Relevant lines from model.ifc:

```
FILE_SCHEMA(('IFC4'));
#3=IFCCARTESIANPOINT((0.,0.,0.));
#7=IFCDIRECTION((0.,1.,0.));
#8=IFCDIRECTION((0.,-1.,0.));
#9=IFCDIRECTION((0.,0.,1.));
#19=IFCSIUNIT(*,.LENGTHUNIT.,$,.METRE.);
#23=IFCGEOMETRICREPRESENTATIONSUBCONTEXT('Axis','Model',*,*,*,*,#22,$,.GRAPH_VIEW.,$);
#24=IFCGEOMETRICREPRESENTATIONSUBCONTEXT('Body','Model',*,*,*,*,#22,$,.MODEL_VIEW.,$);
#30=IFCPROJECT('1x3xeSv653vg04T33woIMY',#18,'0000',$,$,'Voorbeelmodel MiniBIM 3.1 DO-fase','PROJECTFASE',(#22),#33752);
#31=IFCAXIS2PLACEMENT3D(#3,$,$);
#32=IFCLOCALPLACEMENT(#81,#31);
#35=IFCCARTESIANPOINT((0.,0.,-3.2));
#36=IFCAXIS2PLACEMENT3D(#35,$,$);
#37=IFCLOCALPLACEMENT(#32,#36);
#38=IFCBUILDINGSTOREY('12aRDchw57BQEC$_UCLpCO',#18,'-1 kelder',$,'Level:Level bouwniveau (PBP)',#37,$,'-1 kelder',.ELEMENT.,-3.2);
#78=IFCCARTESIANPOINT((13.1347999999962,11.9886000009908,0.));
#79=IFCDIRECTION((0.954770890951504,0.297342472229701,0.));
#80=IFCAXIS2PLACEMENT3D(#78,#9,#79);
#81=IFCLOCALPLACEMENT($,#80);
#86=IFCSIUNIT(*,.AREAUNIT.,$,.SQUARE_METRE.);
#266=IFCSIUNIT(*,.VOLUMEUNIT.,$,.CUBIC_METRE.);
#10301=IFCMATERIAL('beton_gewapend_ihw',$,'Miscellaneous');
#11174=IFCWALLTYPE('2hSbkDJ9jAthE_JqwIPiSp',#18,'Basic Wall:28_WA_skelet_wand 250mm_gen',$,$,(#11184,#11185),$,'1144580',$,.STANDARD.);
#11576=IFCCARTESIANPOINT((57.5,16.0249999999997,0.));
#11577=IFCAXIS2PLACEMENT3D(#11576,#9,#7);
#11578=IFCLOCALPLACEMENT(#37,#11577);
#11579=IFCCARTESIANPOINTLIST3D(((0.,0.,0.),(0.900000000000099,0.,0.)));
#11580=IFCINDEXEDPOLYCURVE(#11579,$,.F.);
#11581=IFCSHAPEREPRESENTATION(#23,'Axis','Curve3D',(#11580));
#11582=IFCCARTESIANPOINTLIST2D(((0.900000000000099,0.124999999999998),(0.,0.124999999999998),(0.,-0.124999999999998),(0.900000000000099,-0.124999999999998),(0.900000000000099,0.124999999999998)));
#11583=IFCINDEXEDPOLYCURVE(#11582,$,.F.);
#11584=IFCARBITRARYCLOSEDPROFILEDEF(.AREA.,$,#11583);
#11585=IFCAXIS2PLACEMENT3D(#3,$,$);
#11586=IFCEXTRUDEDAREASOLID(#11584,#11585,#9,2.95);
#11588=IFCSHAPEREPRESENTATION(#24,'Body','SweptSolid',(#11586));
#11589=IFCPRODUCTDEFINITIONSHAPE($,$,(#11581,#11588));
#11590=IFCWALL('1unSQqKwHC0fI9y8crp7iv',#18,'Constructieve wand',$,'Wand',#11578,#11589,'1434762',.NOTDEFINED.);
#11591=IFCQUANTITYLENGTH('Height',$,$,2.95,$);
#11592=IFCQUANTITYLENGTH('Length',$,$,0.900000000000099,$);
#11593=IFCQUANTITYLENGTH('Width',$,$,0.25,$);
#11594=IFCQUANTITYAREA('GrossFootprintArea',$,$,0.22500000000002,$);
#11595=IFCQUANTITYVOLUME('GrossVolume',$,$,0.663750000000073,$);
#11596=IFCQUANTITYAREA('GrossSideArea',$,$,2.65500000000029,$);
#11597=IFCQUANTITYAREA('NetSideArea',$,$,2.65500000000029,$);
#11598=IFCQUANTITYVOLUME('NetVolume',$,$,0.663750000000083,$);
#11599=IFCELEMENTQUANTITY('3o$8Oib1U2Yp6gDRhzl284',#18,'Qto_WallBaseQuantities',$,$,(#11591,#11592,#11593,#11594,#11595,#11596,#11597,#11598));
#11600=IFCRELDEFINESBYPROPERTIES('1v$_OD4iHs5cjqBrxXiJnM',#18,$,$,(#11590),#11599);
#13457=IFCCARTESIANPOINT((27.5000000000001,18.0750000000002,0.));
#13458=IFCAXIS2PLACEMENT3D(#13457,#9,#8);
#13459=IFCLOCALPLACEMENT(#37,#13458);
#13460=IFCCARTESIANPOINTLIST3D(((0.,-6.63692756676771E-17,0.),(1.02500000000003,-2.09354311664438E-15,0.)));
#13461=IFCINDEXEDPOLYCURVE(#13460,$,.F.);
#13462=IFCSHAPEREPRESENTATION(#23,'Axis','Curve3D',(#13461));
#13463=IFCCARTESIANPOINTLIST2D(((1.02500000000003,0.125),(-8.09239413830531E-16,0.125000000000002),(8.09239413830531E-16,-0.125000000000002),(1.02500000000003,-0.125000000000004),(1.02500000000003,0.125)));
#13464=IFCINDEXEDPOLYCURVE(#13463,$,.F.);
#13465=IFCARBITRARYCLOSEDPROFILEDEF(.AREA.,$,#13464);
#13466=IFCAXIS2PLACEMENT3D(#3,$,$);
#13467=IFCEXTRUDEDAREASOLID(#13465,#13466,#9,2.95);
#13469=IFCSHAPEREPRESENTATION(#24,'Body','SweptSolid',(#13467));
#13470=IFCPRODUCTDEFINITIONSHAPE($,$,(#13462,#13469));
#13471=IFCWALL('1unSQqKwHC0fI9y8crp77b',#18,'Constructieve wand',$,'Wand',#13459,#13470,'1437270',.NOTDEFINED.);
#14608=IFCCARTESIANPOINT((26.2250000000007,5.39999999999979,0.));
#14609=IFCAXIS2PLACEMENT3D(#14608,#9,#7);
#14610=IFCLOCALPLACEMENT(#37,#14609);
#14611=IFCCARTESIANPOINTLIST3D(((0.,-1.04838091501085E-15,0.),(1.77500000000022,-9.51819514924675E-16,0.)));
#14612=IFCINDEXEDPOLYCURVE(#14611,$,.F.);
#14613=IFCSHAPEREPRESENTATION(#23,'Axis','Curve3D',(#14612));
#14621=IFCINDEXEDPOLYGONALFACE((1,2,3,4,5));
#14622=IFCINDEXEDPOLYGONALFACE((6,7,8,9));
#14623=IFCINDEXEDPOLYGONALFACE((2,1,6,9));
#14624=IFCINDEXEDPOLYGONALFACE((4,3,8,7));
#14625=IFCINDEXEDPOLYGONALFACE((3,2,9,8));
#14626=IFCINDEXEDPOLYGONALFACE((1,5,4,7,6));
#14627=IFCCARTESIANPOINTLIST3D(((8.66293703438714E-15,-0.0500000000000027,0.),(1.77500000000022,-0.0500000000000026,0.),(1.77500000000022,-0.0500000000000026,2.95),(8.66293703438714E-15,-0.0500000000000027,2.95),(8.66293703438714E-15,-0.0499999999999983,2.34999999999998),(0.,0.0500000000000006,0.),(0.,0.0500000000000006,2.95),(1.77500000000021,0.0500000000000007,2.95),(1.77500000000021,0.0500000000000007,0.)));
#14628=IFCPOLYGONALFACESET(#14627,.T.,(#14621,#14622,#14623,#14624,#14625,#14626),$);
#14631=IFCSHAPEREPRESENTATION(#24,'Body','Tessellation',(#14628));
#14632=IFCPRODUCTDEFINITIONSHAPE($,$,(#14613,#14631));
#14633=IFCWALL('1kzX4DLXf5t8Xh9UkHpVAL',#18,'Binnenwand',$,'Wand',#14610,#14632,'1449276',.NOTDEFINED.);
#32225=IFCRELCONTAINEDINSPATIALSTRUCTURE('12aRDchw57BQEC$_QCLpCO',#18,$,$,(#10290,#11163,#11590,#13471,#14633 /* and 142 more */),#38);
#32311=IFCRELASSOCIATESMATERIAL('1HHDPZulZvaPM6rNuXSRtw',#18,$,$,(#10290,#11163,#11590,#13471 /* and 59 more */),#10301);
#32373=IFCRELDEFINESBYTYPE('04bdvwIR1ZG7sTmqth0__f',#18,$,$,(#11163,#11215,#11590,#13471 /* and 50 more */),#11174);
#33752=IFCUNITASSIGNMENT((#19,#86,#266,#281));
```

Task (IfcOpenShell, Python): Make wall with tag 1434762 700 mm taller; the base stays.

```python
import ifcopenshell
import ifcopenshell.api.pset
import ifcopenshell.geom
import ifcopenshell.util.element
import ifcopenshell.util.representation
import ifcopenshell.util.shape
import ifcopenshell.util.unit

model = ifcopenshell.open("model.ifc")
unit_scale = ifcopenshell.util.unit.calculate_unit_scale(model)
area_scale = ifcopenshell.util.unit.calculate_unit_scale(model, "AREAUNIT")
volume_scale = ifcopenshell.util.unit.calculate_unit_scale(model, "VOLUMEUNIT")
settings = ifcopenshell.geom.settings()


def volume(element):
    """Net volume in cubic metres, openings subtracted."""
    shape = ifcopenshell.geom.create_shape(settings, element)
    return ifcopenshell.util.shape.get_volume(shape.geometry)


wall = model.by_guid("1unSQqKwHC0fI9y8crp7iv")
before = volume(wall)

body = ifcopenshell.util.representation.get_representation(wall, "Model", "Body")
solid = body.Items[0]
old_height = solid.Depth
solid.Depth += 0.7
after = volume(wall)
thickness = 0.25  # wall thickness in metres

# Update the stored height, areas and volumes.
qto = model.by_id(ifcopenshell.util.element.get_pset(wall, "Qto_WallBaseQuantities", should_inherit=False)["id"])
ifcopenshell.api.pset.edit_qto(model, qto=qto, properties={
    "Height": solid.Depth,
    "GrossVolume": ifcopenshell.util.element.get_pset(wall, "Qto_WallBaseQuantities", "GrossVolume") * solid.Depth / old_height,
    "GrossSideArea": ifcopenshell.util.element.get_pset(wall, "Qto_WallBaseQuantities", "GrossSideArea") * solid.Depth / old_height,
    "NetSideArea": after / thickness / area_scale,
    "NetVolume": after / volume_scale,
})

print(f"height {old_height:g} -> {solid.Depth:g}, volume {before:.3f} -> {after:.3f} m3")

model.write("model_updated.ifc")
```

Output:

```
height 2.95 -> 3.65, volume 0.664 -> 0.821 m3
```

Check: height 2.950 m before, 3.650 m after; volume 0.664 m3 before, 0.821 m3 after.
